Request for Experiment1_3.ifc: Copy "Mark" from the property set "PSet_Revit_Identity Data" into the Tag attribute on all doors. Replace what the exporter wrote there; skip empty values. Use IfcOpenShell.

First a look at what the model holds.

```python
import ifcopenshell
import ifcopenshell.util.element

model = ifcopenshell.open("Experiment1_3.ifc")
print(model.schema)
doors = model.by_type("IfcDoor")
print(len(doors), "doors")
for e in doors[:8]:
    source = ifcopenshell.util.element.get_pset(e, "PSet_Revit_Identity Data", "Mark")
    target = e.Tag
    print(e.id(), repr(source), repr(target), sep=" | ")
```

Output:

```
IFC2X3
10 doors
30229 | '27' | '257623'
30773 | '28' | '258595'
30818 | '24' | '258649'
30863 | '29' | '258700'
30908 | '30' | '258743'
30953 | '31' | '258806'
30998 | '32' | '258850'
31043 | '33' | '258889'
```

```python
import ifcopenshell
import ifcopenshell.util.element

model = ifcopenshell.open("Experiment1_3.ifc")

count = 0
for e in model.by_type("IfcDoor"):
    value = ifcopenshell.util.element.get_pset(e, "PSet_Revit_Identity Data", "Mark")
    current = e.Tag
    if not value or not value.strip() or current == value:
        continue
    e.Tag = value
    count += 1

print(count, "doors updated")

model.write("Experiment1_3_rev.ifc")
```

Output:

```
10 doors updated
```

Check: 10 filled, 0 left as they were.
